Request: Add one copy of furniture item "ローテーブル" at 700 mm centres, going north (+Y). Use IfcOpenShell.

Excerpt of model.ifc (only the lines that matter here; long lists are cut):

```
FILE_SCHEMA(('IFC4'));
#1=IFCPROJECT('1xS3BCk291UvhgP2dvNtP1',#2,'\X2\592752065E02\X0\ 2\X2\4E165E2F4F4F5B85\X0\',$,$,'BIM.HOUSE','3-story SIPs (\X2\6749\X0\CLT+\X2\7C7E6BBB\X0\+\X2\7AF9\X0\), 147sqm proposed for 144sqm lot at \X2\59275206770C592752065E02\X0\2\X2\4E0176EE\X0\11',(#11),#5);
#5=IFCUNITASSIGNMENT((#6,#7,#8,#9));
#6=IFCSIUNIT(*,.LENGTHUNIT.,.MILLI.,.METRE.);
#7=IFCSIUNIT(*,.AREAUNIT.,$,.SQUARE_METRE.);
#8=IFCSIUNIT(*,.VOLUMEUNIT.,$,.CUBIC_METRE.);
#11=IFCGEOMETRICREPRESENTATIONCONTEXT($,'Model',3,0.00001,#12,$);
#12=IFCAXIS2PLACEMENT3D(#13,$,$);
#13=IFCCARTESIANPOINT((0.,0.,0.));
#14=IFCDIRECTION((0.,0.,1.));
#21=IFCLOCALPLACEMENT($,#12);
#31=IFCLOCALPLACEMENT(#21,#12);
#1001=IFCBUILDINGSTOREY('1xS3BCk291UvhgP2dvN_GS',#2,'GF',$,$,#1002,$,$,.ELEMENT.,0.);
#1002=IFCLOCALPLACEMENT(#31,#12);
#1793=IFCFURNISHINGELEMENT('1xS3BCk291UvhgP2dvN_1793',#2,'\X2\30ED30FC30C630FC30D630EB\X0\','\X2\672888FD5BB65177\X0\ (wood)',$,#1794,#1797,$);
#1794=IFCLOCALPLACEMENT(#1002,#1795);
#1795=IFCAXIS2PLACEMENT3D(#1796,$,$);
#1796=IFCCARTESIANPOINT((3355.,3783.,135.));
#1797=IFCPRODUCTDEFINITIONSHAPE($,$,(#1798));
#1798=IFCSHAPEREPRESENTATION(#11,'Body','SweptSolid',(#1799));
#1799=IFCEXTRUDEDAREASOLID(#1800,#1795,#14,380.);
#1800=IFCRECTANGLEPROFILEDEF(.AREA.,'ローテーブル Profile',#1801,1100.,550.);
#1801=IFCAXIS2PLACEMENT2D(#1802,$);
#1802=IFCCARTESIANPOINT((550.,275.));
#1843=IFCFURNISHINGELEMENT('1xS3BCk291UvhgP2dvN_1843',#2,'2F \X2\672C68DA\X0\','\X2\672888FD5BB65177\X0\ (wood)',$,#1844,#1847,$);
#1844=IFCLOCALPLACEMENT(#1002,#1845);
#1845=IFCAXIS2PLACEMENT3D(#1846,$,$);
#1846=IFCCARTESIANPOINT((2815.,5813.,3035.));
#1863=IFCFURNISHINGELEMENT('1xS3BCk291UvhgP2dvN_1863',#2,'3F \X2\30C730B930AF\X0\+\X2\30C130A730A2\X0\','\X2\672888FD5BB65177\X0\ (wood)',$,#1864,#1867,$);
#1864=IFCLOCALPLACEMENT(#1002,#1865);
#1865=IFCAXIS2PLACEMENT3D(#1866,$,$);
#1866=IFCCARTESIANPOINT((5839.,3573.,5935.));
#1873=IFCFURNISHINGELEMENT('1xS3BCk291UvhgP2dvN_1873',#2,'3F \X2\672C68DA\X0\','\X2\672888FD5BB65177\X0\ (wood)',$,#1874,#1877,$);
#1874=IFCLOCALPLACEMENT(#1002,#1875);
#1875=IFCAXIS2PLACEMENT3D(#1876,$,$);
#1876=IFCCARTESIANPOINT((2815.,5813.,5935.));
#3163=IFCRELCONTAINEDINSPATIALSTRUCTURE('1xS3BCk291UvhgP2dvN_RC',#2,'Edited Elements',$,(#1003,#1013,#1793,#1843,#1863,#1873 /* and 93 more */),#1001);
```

```python
import numpy as np
import ifcopenshell
import ifcopenshell.api.geometry
import ifcopenshell.api.root
import ifcopenshell.util.element
import ifcopenshell.util.placement
import ifcopenshell.util.unit

model = ifcopenshell.open("model.ifc")
unit_scale = ifcopenshell.util.unit.calculate_unit_scale(model)


def reuse_history(source, copy):
    """copy_class also copies each property set's owner history, people and application; keep the originals."""
    for rel in copy.IsDefinedBy:
        if rel.is_a("IfcRelDefinesByProperties") and (history := rel.RelatingPropertyDefinition.OwnerHistory):
            rel.RelatingPropertyDefinition.OwnerHistory = source.OwnerHistory
            ifcopenshell.util.element.remove_deep2(model, history)


source = model.by_id(1793)
base = ifcopenshell.util.placement.get_local_placement(source.ObjectPlacement)
step = np.array([0.0, 1.0, 0.0]) * 0.7 / unit_scale

for i in range(1, 2):
    copy = ifcopenshell.api.root.copy_class(model, product=source)
    copy.Representation = ifcopenshell.util.element.copy_deep(
        model, source.Representation, exclude=["IfcGeometricRepresentationContext", "IfcRepresentationMap"]
    )
    reuse_history(source, copy)
    matrix = base.copy()
    matrix[:3, 3] += i * step
    print("added at", matrix[:3, 3].round(3) + 0.0)
    ifcopenshell.api.geometry.edit_object_placement(model, product=copy, matrix=matrix, is_si=False)

model.write("model_rev.ifc")
```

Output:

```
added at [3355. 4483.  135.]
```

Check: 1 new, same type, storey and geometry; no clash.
